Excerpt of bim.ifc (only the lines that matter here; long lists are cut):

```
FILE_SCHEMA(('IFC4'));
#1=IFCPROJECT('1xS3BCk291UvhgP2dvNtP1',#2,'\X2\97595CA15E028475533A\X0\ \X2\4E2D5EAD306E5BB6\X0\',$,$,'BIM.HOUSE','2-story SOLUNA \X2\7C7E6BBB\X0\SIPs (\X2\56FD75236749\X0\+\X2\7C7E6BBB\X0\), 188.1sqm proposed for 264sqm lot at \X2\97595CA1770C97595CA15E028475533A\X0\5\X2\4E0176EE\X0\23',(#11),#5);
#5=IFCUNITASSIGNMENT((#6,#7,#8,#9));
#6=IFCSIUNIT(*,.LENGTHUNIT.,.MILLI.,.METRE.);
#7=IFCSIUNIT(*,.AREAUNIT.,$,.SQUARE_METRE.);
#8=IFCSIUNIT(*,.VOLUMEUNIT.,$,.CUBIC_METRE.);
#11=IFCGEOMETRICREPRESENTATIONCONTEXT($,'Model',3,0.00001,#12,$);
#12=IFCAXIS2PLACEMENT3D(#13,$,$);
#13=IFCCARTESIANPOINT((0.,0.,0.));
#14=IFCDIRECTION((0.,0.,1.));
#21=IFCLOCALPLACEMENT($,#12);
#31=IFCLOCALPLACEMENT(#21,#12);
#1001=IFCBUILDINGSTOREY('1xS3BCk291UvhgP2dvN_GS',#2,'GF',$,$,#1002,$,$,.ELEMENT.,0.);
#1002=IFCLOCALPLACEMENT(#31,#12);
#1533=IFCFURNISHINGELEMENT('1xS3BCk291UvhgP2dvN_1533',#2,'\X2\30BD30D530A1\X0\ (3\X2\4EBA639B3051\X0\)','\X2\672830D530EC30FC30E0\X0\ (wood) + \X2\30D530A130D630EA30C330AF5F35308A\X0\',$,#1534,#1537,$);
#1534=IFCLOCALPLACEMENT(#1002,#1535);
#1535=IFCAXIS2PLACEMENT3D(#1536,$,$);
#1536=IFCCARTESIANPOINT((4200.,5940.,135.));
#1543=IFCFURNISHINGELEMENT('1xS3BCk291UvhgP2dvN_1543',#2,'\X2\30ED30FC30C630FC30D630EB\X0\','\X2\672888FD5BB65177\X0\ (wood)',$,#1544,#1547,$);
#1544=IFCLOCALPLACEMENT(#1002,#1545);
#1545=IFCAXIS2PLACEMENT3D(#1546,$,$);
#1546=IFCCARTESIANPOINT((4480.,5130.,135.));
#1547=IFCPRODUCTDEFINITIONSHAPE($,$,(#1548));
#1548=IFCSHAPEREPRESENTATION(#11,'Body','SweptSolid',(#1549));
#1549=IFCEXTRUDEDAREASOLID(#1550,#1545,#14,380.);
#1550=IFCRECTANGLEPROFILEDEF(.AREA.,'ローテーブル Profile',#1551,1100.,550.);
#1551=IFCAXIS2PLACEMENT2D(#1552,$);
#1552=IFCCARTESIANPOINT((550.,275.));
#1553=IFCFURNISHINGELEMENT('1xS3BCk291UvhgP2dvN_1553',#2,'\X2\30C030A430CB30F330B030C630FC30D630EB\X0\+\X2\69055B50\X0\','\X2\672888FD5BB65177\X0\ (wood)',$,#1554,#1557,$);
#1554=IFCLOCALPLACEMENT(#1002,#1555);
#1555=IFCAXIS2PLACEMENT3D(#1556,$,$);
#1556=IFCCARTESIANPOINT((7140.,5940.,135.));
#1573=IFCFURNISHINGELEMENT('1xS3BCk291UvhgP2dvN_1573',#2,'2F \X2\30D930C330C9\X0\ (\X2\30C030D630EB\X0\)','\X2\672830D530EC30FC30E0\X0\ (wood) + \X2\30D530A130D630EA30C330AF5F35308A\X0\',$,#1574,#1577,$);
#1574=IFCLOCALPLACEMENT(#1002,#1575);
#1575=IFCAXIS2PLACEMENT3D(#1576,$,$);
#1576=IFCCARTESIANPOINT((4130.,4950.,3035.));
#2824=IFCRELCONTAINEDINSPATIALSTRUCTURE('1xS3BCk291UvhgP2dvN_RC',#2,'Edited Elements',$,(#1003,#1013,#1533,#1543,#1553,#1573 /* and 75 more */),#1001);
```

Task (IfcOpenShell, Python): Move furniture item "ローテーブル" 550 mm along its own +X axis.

```python
import ifcopenshell
import ifcopenshell.api.geometry
import ifcopenshell.util.placement

model = ifcopenshell.open("bim.ifc")

item = model.by_guid("1xS3BCk291UvhgP2dvN_1543")
matrix = ifcopenshell.util.placement.get_local_placement(item.ObjectPlacement)
matrix[:3, 3] += matrix[:3, 0] * 550.0
ifcopenshell.api.geometry.edit_object_placement(model, product=item, matrix=matrix, is_si=False)

print(ifcopenshell.util.placement.get_local_placement(item.ObjectPlacement).round(3) + 0.0)

model.write("bim_edited.ifc")
```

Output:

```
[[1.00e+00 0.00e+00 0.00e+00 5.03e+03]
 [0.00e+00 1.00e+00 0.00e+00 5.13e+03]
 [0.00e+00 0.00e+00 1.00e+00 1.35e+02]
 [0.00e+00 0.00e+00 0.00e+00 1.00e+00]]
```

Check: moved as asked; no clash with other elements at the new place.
